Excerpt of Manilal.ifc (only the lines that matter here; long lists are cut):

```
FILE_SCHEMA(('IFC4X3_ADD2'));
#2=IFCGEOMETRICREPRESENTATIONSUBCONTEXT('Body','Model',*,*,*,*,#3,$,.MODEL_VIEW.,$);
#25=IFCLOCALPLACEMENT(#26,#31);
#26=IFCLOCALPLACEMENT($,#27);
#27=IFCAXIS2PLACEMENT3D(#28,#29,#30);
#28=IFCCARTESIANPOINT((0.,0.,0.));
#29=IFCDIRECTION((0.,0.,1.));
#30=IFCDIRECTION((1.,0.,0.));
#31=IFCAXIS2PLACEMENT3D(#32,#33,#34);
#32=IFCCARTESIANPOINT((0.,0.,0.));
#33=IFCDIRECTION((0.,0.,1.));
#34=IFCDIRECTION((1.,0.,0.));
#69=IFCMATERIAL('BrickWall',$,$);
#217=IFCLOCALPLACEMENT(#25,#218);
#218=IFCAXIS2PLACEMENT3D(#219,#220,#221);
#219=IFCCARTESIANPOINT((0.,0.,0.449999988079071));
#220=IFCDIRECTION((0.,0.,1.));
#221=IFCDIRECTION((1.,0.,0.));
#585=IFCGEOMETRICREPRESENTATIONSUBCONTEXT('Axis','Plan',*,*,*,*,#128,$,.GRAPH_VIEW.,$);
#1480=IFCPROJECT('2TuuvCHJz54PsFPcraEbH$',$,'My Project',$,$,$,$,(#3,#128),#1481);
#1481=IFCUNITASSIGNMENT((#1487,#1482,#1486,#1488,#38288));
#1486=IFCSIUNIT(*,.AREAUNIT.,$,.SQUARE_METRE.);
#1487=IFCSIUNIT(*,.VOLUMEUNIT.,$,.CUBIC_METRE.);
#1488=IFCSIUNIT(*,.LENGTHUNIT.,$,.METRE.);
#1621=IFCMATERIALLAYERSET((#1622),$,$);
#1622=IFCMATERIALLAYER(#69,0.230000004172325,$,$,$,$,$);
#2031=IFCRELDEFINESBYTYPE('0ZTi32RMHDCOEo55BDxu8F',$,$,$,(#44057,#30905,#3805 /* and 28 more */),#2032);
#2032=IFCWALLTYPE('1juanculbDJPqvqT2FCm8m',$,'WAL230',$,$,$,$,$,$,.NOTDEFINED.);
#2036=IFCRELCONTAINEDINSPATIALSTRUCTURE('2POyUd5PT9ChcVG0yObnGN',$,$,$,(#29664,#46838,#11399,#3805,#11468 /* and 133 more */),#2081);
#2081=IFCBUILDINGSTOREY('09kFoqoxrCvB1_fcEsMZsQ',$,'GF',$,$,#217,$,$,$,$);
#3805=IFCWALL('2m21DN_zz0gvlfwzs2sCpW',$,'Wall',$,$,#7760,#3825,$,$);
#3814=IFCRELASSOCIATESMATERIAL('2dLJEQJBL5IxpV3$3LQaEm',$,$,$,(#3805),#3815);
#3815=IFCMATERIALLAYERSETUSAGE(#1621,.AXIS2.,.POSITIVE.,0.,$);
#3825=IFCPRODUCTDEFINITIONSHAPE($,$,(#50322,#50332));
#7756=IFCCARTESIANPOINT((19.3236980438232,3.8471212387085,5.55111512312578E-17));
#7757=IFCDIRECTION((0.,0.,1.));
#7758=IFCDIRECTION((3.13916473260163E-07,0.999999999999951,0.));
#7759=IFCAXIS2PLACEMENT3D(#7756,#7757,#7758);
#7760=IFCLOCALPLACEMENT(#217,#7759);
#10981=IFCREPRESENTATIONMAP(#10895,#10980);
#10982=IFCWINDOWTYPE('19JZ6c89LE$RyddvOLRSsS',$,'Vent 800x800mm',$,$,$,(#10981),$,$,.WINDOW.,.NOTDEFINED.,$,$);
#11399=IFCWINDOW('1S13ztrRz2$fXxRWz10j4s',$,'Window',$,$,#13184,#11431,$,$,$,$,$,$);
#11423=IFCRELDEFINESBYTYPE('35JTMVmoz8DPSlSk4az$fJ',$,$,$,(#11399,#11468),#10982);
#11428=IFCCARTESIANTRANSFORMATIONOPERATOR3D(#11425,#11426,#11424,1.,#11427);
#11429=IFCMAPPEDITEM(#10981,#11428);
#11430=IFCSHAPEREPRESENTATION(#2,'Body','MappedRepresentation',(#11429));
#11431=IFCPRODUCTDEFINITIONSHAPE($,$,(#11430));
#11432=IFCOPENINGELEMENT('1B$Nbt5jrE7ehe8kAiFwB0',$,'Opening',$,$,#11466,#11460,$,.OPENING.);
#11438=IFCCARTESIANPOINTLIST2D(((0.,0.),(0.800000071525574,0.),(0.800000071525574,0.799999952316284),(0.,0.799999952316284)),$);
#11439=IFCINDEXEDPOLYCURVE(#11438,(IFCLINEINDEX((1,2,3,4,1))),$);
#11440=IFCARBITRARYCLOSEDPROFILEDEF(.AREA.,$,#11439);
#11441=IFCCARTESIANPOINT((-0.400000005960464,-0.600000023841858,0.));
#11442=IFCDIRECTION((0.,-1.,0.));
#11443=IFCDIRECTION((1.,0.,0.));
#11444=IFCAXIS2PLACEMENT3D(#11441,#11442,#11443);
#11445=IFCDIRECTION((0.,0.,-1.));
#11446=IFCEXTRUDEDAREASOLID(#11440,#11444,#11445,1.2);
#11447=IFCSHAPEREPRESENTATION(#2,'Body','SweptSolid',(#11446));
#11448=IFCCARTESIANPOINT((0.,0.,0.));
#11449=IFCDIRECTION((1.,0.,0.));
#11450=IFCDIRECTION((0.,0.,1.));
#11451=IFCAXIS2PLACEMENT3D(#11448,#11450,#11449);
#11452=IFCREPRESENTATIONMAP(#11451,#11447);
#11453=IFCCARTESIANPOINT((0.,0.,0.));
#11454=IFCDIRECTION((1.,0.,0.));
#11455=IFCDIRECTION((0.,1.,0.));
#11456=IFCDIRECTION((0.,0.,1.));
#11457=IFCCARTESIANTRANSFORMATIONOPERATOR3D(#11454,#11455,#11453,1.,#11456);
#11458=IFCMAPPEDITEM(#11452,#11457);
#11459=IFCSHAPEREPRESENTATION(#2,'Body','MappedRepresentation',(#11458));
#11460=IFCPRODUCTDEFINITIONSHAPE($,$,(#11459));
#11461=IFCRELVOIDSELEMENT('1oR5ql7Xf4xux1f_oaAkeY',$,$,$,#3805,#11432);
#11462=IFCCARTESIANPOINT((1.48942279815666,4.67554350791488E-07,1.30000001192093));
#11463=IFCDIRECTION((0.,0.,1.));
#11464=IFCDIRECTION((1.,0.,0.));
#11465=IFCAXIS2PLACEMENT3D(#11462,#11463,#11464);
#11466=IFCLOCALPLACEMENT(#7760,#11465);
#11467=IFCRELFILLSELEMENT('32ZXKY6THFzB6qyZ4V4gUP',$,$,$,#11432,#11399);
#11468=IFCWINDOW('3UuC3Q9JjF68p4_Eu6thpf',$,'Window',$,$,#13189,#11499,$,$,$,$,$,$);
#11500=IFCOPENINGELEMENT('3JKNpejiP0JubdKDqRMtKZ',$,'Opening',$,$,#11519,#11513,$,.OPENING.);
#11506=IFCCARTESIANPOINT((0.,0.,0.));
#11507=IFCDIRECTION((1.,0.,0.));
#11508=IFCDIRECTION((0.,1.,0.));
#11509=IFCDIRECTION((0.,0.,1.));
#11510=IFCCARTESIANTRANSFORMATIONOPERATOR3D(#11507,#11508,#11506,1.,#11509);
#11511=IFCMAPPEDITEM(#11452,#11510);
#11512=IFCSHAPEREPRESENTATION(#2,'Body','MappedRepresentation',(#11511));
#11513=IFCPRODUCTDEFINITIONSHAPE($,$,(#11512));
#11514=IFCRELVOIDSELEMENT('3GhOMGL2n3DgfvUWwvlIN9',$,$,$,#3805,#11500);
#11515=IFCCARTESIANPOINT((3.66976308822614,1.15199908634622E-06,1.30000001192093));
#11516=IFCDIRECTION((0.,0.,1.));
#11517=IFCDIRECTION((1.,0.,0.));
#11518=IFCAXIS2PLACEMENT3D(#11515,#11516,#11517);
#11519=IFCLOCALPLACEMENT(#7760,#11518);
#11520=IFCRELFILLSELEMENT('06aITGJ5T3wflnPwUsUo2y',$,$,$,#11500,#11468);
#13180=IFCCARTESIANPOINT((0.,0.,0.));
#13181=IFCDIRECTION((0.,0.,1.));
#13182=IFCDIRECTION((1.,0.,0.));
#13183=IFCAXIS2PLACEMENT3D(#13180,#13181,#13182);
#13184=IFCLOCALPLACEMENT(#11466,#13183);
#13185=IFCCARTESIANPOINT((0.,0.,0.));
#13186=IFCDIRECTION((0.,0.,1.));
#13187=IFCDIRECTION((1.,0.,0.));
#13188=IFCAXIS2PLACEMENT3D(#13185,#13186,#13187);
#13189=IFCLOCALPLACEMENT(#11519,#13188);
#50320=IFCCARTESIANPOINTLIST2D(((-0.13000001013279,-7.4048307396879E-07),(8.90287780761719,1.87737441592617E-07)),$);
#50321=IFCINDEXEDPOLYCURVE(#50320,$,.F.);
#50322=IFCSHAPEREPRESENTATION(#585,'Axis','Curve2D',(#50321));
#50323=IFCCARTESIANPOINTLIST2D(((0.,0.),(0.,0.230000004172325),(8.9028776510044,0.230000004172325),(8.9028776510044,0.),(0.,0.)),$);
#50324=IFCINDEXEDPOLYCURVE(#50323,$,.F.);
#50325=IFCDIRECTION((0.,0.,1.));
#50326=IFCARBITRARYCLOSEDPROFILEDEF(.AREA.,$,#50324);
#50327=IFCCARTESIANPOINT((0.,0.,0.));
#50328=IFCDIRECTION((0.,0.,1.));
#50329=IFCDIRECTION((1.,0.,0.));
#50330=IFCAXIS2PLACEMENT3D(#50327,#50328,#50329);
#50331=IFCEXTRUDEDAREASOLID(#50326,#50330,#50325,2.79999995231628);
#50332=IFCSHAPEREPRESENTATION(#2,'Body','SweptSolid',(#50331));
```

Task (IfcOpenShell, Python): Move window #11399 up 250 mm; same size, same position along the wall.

```python
import numpy as np
import ifcopenshell
import ifcopenshell.api.geometry
import ifcopenshell.util.placement
import ifcopenshell.util.unit

model = ifcopenshell.open("Manilal.ifc")
unit_scale = ifcopenshell.util.unit.calculate_unit_scale(model)

window = model.by_guid("1S13ztrRz2$fXxRWz10j4s")
opening = window.FillsVoids[0].RelatingOpeningElement
dz = 0.25 / unit_scale

shift = np.array([0.0, 0.0, dz])
# The window is placed relative to its opening, so it follows when the opening moves.
matrix = ifcopenshell.util.placement.get_local_placement(opening.ObjectPlacement)
matrix[:3, 3] += shift
ifcopenshell.api.geometry.edit_object_placement(
    model, product=opening, matrix=matrix, is_si=False, should_transform_children=True
)

print(f"moved by {dz * unit_scale:+.3f} m")

model.write("Manilal_rev.ifc")
```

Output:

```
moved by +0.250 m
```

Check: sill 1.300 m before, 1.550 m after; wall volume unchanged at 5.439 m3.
